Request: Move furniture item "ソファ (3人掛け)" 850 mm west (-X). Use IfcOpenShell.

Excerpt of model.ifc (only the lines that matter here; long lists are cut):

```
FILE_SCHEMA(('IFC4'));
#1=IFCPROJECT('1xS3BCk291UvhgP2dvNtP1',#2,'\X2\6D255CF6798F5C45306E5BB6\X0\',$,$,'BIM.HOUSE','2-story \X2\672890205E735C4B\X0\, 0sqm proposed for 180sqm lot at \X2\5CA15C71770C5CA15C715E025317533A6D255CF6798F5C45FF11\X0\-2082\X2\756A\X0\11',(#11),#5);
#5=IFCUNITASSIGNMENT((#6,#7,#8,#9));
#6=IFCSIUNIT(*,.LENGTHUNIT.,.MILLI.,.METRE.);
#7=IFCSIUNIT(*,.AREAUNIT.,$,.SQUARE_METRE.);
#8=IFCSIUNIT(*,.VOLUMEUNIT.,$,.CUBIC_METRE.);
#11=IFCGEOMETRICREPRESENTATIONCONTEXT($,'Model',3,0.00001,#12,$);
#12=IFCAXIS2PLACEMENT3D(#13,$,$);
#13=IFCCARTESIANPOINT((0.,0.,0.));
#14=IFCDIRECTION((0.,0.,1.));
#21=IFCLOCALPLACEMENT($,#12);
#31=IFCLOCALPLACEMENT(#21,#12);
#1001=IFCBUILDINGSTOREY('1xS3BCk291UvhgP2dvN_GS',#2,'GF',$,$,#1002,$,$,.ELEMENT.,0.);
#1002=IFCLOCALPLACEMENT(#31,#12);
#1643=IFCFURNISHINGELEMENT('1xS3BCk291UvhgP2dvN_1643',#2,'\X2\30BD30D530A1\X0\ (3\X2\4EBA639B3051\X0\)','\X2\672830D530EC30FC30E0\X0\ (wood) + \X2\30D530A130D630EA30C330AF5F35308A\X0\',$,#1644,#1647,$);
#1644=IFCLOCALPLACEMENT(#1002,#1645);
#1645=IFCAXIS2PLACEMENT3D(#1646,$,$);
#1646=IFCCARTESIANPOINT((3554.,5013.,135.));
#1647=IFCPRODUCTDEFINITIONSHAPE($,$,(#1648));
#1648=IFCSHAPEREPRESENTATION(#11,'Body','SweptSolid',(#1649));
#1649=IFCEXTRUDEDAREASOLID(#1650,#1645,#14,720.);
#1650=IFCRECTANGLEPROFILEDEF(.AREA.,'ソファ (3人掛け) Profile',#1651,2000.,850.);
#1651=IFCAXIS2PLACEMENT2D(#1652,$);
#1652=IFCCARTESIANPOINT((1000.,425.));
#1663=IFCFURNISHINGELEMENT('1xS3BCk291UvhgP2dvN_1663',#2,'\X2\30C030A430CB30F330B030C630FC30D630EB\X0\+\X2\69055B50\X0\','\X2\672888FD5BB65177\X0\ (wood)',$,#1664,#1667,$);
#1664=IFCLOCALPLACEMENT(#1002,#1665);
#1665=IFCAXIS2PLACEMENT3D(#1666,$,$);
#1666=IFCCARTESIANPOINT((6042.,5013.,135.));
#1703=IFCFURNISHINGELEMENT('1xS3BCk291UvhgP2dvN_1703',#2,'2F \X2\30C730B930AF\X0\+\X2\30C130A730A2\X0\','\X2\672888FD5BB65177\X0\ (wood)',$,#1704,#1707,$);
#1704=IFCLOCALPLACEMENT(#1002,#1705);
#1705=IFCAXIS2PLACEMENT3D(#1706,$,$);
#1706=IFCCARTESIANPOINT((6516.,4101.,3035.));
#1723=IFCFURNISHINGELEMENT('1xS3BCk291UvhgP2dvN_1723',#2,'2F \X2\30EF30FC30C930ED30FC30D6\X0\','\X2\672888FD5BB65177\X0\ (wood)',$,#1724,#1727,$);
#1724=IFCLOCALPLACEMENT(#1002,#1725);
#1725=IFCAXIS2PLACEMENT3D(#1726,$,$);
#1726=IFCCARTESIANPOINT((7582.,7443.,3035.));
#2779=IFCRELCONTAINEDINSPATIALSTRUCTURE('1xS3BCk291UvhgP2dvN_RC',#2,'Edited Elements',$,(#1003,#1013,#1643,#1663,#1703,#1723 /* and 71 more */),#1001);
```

```python
import ifcopenshell
import ifcopenshell.api.geometry
import ifcopenshell.util.placement
import ifcopenshell.util.unit

model = ifcopenshell.open("model.ifc")
unit_scale = ifcopenshell.util.unit.calculate_unit_scale(model)

item = model.by_guid("1xS3BCk291UvhgP2dvN_1643")
matrix = ifcopenshell.util.placement.get_local_placement(item.ObjectPlacement)
matrix[0, 3] -= 0.85 / unit_scale
ifcopenshell.api.geometry.edit_object_placement(model, product=item, matrix=matrix, is_si=False)

print(ifcopenshell.util.placement.get_local_placement(item.ObjectPlacement).round(3) + 0.0)

model.write("model_v2.ifc")
```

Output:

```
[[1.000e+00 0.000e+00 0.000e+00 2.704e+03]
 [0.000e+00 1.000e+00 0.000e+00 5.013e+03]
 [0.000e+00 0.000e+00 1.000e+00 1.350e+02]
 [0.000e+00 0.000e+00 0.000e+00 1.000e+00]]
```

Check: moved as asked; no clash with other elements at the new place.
